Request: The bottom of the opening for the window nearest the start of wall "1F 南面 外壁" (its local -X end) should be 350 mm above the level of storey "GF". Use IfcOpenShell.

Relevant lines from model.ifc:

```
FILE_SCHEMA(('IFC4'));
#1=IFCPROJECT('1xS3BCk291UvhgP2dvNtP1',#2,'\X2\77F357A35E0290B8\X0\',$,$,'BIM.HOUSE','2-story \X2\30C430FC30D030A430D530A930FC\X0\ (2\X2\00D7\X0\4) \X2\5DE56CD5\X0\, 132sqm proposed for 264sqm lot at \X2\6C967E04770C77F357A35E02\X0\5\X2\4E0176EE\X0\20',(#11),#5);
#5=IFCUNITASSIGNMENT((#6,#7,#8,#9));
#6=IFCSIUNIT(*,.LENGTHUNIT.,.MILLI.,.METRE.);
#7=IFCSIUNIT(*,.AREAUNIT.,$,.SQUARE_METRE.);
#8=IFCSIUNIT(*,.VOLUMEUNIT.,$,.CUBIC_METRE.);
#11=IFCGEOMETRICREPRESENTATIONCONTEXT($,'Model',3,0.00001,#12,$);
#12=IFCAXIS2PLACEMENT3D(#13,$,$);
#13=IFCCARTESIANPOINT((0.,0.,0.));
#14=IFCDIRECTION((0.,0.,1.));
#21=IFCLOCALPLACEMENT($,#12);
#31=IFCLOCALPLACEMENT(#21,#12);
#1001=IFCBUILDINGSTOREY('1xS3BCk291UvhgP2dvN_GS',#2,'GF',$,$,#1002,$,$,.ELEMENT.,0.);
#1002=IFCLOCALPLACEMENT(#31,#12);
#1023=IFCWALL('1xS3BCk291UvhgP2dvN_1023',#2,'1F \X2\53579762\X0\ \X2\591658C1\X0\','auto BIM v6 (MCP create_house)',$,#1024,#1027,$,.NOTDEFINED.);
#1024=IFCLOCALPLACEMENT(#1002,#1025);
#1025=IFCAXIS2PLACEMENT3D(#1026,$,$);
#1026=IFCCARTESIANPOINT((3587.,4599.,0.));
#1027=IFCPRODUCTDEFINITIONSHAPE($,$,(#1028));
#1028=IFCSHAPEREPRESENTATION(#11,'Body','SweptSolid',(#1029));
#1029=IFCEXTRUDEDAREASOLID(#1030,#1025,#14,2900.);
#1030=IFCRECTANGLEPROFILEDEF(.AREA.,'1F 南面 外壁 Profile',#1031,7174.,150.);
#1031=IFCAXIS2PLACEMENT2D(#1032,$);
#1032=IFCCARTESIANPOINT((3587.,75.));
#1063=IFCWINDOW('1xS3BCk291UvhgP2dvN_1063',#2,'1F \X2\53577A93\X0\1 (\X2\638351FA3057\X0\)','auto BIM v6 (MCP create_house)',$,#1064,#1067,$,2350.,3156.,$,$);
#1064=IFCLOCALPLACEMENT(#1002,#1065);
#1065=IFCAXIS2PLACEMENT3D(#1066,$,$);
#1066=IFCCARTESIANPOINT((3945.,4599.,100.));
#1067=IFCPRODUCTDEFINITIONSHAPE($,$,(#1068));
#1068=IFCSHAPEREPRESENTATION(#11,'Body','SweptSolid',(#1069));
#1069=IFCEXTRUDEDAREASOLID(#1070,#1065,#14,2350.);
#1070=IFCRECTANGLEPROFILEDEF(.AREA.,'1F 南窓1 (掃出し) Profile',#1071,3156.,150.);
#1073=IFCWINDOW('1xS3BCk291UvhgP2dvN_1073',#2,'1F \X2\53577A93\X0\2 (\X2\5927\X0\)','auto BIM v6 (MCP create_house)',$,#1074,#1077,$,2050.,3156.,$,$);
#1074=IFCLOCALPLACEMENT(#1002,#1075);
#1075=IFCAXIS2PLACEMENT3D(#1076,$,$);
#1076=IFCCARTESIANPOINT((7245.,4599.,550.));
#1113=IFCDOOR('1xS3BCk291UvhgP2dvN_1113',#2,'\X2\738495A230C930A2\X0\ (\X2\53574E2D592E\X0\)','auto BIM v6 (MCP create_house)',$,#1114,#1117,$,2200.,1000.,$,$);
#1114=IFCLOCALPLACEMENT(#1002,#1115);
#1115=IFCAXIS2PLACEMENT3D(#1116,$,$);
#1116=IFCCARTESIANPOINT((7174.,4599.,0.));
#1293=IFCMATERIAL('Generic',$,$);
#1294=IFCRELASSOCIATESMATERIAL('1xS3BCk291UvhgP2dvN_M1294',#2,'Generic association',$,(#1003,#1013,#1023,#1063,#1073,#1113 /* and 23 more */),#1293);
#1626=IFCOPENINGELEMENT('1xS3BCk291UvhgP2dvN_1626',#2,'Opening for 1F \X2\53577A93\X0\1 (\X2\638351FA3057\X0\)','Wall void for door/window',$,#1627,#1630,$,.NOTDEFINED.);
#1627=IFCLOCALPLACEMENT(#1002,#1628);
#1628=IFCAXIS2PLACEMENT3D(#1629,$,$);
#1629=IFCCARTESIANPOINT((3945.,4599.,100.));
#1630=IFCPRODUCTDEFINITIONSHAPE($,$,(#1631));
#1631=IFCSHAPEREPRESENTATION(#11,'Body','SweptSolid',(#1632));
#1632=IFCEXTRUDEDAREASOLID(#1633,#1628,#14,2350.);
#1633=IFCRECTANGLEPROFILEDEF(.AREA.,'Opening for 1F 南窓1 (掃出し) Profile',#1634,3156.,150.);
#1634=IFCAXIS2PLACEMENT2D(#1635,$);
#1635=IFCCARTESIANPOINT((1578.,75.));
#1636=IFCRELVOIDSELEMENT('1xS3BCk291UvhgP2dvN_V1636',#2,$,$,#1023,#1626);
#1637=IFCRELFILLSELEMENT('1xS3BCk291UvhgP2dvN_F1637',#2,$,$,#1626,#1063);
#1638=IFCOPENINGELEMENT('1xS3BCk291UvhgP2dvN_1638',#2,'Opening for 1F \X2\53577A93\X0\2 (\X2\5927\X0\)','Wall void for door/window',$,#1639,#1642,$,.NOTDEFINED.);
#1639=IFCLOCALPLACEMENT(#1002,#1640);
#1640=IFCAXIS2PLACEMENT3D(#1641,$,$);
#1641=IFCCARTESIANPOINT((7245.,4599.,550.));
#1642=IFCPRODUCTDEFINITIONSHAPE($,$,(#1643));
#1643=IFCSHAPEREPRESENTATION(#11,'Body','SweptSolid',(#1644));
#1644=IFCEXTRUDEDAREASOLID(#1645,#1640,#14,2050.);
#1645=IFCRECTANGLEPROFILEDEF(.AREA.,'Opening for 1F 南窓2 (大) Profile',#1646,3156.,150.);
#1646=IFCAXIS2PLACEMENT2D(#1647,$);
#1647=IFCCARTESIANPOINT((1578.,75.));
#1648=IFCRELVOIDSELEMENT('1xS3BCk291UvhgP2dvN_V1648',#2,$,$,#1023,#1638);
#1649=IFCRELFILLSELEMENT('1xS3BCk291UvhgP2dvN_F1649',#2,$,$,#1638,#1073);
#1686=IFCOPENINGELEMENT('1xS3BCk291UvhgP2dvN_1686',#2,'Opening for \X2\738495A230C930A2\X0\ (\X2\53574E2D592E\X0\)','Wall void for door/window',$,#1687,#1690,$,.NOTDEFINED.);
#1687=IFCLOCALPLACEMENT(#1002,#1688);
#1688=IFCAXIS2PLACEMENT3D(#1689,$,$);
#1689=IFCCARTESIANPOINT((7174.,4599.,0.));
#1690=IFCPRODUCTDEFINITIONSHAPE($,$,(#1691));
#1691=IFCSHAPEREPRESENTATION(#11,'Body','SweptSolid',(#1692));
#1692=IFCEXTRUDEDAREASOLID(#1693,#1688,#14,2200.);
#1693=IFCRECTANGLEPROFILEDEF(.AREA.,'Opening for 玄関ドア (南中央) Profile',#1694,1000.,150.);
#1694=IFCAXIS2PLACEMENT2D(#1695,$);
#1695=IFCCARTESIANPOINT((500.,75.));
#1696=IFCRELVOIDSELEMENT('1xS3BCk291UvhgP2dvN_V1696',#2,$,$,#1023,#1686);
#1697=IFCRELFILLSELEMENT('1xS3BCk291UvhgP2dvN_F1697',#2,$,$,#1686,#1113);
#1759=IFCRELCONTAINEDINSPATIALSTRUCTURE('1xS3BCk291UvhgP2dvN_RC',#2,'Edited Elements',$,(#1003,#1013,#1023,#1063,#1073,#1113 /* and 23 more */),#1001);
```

```python
import numpy as np
import ifcopenshell
import ifcopenshell.api.geometry
import ifcopenshell.geom
import ifcopenshell.util.element
import ifcopenshell.util.placement
import ifcopenshell.util.shape
import ifcopenshell.util.unit

model = ifcopenshell.open("model.ifc")
unit_scale = ifcopenshell.util.unit.calculate_unit_scale(model)

window = model.by_id(1063)
opening = window.FillsVoids[0].RelatingOpeningElement
storey = ifcopenshell.util.element.get_container(window, ifc_class="IfcBuildingStorey")
level = ifcopenshell.util.placement.get_local_placement(storey.ObjectPlacement)[2, 3]

# The opening's origin need not be at the sill, so measure its lowest point.
shape = ifcopenshell.geom.create_shape(ifcopenshell.geom.settings(), opening)
bottom = ifcopenshell.util.shape.get_shape_bottom_elevation(shape, shape.geometry) / unit_scale
dz = level + 350.0 - bottom

shift = np.array([0.0, 0.0, dz])
# The window is not placed relative to its opening, so move both.
for product in (opening, window):
    matrix = ifcopenshell.util.placement.get_local_placement(product.ObjectPlacement)
    matrix[:3, 3] += shift
    ifcopenshell.api.geometry.edit_object_placement(model, product=product, matrix=matrix, is_si=False)

print(f"moved by {dz * unit_scale:+.3f} m")

model.write("model_updated.ifc")
```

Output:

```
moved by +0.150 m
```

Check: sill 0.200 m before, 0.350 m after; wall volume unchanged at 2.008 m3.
